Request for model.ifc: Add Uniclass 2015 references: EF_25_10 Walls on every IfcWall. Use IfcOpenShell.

First a look at what the model holds.

```python
import ifcopenshell

model = ifcopenshell.open("model.ifc")
print(model.schema)
print("classifications:", [c.Name for c in model.by_type("IfcClassification")])
for ifc_class in ("IfcDoor", "IfcRoof", "IfcStair", "IfcWall", "IfcWindow"):
    print(ifc_class, len(model.by_type(ifc_class)))
```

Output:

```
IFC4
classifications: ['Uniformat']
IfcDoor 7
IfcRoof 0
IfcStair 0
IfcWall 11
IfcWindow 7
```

```python
import ifcopenshell
import ifcopenshell.api.classification

model = ifcopenshell.open("model.ifc")

system = ifcopenshell.api.classification.add_classification(model, classification="Uniclass 2015")

codes = {
    "IfcWall": ("EF_25_10", "Walls"),
}
for ifc_class, (code, name) in codes.items():
    products = model.by_type(ifc_class)
    ifcopenshell.api.classification.add_reference(
        model, products=products, classification=system, identification=code, name=name
    )
    print(code, len(products))

model.write("model-out.ifc")
```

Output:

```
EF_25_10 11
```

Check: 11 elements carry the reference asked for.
